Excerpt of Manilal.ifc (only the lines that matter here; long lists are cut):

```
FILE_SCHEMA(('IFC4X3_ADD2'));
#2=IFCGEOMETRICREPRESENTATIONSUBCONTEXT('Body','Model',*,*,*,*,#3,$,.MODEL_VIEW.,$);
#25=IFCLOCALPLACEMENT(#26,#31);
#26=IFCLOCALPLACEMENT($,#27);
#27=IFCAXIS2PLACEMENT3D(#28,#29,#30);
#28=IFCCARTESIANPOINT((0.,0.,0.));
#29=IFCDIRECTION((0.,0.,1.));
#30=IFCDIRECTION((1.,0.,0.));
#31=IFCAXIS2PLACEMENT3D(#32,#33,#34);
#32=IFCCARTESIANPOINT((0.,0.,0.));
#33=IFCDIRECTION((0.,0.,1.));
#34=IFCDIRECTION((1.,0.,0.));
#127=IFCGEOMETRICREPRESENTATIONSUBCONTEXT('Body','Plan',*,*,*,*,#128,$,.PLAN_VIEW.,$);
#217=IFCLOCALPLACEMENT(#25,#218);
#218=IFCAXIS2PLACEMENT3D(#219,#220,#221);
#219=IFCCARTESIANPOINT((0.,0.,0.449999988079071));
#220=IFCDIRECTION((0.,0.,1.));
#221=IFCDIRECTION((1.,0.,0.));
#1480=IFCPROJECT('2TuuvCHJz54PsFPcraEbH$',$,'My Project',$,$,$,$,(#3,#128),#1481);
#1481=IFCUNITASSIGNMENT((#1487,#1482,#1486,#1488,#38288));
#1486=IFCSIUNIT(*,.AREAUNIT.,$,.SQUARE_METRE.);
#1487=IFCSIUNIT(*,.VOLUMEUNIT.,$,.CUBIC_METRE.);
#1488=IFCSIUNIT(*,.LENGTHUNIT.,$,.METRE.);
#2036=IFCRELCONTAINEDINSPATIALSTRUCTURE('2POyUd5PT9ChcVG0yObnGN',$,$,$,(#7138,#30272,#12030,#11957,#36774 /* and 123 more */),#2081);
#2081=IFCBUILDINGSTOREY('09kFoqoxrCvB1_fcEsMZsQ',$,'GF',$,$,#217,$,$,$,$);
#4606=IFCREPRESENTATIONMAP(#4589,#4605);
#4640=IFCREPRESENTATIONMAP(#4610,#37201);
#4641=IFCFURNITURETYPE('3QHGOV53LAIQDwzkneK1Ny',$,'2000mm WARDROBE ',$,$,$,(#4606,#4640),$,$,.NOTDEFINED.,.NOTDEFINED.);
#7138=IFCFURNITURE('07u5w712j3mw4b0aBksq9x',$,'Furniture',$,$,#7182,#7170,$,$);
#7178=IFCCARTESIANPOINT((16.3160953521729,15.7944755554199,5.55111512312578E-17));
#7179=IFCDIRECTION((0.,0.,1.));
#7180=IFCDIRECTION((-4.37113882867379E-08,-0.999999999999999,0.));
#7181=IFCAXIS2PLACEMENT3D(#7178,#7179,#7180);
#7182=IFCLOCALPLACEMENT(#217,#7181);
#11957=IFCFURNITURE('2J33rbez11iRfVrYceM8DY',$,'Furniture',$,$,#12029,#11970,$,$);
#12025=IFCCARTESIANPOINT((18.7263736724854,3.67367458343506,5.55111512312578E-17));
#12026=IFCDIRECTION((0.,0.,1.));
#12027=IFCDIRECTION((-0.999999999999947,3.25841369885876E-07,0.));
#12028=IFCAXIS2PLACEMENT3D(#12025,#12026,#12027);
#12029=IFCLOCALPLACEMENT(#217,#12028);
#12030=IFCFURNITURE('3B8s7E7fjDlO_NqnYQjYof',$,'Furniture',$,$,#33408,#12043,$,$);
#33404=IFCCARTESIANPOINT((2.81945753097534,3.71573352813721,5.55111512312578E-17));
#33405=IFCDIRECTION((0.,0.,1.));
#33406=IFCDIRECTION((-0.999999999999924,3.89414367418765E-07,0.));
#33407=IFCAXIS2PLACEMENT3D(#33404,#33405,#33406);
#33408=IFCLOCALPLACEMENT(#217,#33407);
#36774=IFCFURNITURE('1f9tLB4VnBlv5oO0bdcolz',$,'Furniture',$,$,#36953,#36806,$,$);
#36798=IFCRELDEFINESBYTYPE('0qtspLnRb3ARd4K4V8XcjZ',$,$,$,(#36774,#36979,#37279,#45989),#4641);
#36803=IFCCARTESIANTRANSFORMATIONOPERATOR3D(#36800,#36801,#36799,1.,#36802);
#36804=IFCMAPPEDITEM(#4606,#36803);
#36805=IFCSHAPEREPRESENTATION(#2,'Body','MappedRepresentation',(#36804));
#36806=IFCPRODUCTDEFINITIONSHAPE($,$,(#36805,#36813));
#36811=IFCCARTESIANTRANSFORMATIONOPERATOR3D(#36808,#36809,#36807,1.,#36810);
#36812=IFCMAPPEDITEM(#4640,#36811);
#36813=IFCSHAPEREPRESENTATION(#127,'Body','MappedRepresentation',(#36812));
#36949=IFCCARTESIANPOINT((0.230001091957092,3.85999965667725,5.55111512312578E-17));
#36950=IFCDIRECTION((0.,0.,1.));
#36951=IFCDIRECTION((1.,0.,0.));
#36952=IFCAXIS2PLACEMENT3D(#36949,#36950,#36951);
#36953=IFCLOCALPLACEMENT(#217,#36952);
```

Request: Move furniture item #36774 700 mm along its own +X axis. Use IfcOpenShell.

```python
import ifcopenshell
import ifcopenshell.api.geometry
import ifcopenshell.util.placement
import ifcopenshell.util.unit

model = ifcopenshell.open("Manilal.ifc")
unit_scale = ifcopenshell.util.unit.calculate_unit_scale(model)

item = model.by_id(36774)
matrix = ifcopenshell.util.placement.get_local_placement(item.ObjectPlacement)
matrix[:3, 3] += matrix[:3, 0] * 0.7 / unit_scale
ifcopenshell.api.geometry.edit_object_placement(model, product=item, matrix=matrix, is_si=False)

print(ifcopenshell.util.placement.get_local_placement(item.ObjectPlacement).round(3) + 0.0)

model.write("Manilal_updated.ifc")
```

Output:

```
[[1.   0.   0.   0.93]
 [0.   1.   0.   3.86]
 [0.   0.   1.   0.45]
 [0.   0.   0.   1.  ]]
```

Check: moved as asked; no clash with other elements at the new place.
